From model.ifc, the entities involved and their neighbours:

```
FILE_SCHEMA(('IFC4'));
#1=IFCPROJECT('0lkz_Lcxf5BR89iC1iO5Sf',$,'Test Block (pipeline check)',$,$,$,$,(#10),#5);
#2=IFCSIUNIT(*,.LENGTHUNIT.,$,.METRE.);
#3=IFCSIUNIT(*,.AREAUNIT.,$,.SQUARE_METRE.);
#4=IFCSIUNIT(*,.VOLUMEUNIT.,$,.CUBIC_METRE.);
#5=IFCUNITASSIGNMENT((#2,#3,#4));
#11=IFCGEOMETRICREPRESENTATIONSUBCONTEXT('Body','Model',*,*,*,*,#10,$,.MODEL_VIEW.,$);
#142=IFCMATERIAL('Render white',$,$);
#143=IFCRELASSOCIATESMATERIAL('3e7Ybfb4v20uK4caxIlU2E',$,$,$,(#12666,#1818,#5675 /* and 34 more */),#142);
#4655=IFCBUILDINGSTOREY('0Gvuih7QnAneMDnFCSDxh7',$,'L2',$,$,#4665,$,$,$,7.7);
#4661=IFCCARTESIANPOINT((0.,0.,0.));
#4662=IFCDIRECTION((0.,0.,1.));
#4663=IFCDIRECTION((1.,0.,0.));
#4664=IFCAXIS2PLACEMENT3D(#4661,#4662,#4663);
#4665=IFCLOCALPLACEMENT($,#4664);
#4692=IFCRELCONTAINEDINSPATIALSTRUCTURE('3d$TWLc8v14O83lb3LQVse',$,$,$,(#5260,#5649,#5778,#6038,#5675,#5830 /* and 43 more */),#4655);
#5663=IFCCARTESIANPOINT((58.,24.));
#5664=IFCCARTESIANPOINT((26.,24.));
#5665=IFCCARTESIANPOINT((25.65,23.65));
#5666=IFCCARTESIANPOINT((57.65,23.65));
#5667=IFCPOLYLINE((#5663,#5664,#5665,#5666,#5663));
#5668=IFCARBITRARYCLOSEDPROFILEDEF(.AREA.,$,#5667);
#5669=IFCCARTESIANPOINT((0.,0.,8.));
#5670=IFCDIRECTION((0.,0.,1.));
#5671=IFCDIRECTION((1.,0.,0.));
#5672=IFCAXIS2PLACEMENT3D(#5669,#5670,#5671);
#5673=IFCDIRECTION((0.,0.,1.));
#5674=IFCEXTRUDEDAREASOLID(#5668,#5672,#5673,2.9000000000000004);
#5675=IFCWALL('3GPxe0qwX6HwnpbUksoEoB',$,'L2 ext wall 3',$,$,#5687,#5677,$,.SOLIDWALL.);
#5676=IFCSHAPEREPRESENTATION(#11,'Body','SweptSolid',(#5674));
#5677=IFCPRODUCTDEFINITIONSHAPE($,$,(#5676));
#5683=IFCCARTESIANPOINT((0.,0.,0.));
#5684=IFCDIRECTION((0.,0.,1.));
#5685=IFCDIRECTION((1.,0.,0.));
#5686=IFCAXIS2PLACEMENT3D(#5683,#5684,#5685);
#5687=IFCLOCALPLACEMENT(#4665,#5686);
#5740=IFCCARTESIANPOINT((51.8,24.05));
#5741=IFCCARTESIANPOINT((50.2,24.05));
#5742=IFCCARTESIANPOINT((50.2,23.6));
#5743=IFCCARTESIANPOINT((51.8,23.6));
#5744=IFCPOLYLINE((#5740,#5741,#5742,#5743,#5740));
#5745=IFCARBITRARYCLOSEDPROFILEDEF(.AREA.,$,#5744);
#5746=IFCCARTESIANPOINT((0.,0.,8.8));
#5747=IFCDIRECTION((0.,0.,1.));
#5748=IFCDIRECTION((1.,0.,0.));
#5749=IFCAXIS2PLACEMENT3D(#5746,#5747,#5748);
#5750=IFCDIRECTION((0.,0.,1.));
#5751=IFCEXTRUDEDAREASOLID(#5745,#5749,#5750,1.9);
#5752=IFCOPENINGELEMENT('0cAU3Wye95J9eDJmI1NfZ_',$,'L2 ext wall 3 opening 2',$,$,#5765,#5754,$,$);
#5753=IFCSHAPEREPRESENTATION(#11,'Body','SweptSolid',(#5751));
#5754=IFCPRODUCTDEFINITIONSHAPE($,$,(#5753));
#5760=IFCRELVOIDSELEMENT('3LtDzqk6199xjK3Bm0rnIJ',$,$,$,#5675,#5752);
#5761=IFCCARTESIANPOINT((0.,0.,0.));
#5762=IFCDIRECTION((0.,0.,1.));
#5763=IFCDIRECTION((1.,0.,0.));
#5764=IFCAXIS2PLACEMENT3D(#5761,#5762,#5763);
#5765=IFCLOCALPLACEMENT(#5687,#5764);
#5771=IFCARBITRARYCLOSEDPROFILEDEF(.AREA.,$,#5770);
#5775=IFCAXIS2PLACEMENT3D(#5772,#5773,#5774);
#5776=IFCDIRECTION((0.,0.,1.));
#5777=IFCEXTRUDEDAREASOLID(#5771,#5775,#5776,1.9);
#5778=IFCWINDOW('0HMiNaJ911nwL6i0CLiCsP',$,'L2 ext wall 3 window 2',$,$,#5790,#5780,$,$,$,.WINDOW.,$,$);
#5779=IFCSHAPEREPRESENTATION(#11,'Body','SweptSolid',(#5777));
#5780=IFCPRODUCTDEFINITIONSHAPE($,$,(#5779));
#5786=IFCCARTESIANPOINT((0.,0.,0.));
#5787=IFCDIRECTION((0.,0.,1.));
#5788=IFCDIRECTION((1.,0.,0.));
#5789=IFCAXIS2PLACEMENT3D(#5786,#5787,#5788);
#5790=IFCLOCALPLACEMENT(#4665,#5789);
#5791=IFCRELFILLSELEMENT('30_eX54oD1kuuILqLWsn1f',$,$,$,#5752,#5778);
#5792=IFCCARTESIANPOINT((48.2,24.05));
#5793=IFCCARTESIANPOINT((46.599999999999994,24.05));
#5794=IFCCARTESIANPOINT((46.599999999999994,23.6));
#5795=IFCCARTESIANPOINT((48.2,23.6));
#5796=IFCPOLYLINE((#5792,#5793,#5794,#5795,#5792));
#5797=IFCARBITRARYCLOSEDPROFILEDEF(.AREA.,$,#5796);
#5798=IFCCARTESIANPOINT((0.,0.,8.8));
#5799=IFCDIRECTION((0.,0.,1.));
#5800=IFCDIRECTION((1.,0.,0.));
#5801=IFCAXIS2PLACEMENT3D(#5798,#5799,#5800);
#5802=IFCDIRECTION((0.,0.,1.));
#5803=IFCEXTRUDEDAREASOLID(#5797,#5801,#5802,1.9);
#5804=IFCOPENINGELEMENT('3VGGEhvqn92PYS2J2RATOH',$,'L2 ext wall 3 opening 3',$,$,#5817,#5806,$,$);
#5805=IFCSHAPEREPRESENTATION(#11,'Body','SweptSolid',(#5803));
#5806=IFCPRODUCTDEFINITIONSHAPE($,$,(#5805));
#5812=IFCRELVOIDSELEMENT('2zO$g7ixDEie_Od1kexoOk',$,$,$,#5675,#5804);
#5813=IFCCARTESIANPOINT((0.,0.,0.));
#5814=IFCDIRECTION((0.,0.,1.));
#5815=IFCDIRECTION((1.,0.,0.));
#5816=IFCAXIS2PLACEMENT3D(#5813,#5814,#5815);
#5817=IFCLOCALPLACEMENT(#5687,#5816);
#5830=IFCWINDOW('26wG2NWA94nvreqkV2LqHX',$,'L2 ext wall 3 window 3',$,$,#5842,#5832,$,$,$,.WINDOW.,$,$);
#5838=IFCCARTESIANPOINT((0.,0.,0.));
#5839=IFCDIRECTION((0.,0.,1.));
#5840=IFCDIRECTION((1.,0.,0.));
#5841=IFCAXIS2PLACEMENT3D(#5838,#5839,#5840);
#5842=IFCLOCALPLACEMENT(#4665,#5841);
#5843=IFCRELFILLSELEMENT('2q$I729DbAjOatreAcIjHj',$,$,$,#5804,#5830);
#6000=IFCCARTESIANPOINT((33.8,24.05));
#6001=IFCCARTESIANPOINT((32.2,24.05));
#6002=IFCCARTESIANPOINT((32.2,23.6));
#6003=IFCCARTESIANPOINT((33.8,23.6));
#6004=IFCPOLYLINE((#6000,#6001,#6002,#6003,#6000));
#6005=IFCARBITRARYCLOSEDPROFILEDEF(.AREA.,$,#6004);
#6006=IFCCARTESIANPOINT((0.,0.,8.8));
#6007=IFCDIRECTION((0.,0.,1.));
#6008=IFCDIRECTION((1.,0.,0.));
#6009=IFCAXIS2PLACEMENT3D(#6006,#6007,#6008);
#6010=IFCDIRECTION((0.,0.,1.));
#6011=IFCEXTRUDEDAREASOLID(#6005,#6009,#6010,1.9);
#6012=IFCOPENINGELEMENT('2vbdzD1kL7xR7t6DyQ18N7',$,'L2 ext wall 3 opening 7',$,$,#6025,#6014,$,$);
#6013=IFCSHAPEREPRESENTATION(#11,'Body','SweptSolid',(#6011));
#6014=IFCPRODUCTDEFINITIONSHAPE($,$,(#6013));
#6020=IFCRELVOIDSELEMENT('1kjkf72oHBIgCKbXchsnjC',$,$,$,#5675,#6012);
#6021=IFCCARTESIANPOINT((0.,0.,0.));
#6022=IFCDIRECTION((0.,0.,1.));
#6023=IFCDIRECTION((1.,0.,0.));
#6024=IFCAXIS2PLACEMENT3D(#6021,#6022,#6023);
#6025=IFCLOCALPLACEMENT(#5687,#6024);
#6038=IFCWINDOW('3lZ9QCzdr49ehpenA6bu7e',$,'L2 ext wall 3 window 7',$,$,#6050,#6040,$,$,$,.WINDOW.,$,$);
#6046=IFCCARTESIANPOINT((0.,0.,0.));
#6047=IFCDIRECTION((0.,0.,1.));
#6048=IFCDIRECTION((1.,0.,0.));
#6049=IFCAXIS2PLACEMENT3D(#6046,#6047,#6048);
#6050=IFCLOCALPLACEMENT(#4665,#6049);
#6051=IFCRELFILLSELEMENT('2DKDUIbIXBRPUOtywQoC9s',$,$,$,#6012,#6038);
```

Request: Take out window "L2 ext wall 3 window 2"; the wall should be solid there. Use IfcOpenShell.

```python
import ifcopenshell
import ifcopenshell.api.feature
import ifcopenshell.api.root
import ifcopenshell.geom
import ifcopenshell.util.shape

model = ifcopenshell.open("model.ifc")
settings = ifcopenshell.geom.settings()


def volume(element):
    """Net volume in cubic metres, openings subtracted."""
    shape = ifcopenshell.geom.create_shape(settings, element)
    return ifcopenshell.util.shape.get_volume(shape.geometry)


window = model.by_guid("0HMiNaJ911nwL6i0CLiCsP")
opening = window.FillsVoids[0].RelatingOpeningElement
wall = opening.VoidsElements[0].RelatingBuildingElement
before = volume(wall)

ifcopenshell.api.root.remove_product(model, product=window)
ifcopenshell.api.feature.remove_feature(model, feature=opening)

after = volume(wall)

print(f"wall volume {before:.3f} -> {after:.3f} m3")

model.write("model-out.ifc")
```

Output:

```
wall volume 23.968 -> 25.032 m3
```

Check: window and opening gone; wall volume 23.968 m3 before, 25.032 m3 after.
